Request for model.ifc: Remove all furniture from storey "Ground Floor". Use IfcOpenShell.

First a look at what the model holds.

```python
import ifcopenshell
import ifcopenshell.util.element

model = ifcopenshell.open("model.ifc")
print(model.schema)
storey = next(s for s in model.by_type("IfcBuildingStorey") if s.Name == "Ground Floor")
furniture = [e for e in ifcopenshell.util.element.get_decomposition(storey) if e.is_a("IfcFurnishingElement")]
seen = {}
for e in furniture:
    element_type = ifcopenshell.util.element.get_type(e)
    name = element_type.Name if element_type not in (None, e) else None
    seen[name] = seen.get(name, 0) + 1
for name, count in sorted(seen.items(), key=str):
    print(count, "x", name)
```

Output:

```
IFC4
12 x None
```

```python
import ifcopenshell
import ifcopenshell.api.root
import ifcopenshell.util.element

model = ifcopenshell.open("model.ifc")

storey = next(s for s in model.by_type("IfcBuildingStorey") if s.Name == "Ground Floor")
furniture = [e for e in ifcopenshell.util.element.get_decomposition(storey) if e.is_a("IfcFurnishingElement")]

for e in furniture:
    ifcopenshell.api.root.remove_product(model, product=e)
print(len(furniture), "removed")

model.write("model-out.ifc")
```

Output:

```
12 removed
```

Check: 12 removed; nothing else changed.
